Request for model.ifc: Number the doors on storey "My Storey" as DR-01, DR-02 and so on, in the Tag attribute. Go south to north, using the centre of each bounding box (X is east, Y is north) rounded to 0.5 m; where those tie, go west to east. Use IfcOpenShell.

First a look at what the model holds.

```python
import ifcopenshell
import ifcopenshell.util.element
import ifcopenshell.util.placement

model = ifcopenshell.open("model.ifc")
print(model.schema)
storey = next(s for s in model.by_type("IfcBuildingStorey") if s.Name == "My Storey")
doors = [e for e in ifcopenshell.util.element.get_decomposition(storey) if e.is_a("IfcDoor")]
for e in sorted(doors, key=lambda e: e.id()):
    origin = ifcopenshell.util.placement.get_local_placement(e.ObjectPlacement)[:3, 3]
    print(e.id(), e.Tag, e.Name, origin.round(2) + 0.0, sep=" | ")
```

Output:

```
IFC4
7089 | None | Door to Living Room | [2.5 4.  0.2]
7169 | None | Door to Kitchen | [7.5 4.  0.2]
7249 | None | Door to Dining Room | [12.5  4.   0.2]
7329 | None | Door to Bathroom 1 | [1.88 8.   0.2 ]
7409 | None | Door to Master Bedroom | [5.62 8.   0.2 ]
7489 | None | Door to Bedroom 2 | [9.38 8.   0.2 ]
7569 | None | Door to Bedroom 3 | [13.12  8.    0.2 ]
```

```python
import ifcopenshell
import ifcopenshell.geom
import ifcopenshell.util.element
import ifcopenshell.util.shape

model = ifcopenshell.open("model.ifc")
settings = ifcopenshell.geom.settings()
settings.set("use-world-coords", True)


def centre(element):
    shape = ifcopenshell.geom.create_shape(settings, element)
    return ifcopenshell.util.shape.get_bbox_centroid(shape.geometry)


storey = next(s for s in model.by_type("IfcBuildingStorey") if s.Name == "My Storey")
doors = [e for e in ifcopenshell.util.element.get_decomposition(storey) if e.is_a("IfcDoor")]

# Insertion points can sit at a corner or the storey origin, so sort by the geometry (in metres).
centres = {e: centre(e) for e in doors}
doors.sort(key=lambda e: (round(centres[e][1] / 0.5), centres[e][0]))

for i, e in enumerate(doors, start=1):
    number = f"DR-{i:02d}"
    e.Tag = number
    print(e.id(), number)

model.write("model_edited.ifc")
```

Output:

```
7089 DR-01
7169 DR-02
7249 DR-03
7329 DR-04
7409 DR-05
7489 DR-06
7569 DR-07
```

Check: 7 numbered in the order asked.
